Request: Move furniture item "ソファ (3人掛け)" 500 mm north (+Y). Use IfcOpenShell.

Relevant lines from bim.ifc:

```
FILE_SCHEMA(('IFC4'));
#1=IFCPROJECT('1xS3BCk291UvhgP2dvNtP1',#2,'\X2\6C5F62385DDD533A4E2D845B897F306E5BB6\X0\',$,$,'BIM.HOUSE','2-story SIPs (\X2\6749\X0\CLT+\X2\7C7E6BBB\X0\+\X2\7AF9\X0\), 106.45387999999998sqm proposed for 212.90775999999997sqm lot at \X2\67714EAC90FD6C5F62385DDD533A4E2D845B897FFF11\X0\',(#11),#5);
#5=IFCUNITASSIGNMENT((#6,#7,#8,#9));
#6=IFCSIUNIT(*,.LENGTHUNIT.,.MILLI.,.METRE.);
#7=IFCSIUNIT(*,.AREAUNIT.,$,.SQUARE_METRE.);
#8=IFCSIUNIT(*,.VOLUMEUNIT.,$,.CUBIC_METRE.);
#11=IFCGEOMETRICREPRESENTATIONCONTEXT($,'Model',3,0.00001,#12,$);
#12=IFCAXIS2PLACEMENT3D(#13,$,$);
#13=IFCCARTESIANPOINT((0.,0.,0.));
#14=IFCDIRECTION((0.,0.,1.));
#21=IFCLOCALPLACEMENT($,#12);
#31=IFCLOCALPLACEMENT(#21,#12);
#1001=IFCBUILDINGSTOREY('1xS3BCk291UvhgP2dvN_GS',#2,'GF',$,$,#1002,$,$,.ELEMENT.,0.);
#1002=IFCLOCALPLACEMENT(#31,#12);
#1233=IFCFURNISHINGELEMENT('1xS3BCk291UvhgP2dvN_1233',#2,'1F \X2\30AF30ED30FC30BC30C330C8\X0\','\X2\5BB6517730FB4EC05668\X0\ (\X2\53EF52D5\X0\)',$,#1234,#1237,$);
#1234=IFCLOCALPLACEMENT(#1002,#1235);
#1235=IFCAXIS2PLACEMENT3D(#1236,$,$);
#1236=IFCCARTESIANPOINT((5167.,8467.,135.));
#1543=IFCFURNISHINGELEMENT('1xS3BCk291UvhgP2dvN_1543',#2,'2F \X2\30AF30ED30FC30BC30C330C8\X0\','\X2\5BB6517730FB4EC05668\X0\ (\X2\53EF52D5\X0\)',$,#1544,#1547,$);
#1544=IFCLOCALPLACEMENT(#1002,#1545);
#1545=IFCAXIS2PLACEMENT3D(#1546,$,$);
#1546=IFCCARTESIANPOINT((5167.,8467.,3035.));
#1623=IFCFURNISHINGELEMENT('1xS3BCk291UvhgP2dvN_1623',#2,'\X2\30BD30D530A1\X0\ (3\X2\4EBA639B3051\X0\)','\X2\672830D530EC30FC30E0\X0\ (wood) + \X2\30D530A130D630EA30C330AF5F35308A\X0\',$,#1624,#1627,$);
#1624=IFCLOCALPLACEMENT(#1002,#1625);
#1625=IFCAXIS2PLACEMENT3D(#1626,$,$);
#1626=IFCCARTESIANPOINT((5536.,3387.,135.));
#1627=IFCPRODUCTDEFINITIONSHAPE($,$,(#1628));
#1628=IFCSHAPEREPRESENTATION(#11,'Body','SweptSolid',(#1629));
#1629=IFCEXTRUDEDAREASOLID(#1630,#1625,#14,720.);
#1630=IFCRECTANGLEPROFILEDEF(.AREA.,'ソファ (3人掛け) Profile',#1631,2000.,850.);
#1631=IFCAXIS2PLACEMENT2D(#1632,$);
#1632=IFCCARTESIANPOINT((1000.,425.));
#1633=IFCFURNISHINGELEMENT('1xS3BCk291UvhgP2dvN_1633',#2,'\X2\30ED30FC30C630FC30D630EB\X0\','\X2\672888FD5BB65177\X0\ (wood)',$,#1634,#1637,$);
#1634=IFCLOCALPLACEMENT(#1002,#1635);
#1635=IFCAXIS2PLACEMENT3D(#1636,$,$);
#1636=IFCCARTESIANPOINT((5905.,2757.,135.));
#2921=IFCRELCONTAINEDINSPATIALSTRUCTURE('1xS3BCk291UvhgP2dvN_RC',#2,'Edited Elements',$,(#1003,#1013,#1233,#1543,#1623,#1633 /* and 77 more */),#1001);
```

```python
import ifcopenshell
import ifcopenshell.api.geometry
import ifcopenshell.util.placement

model = ifcopenshell.open("bim.ifc")

item = model.by_guid("1xS3BCk291UvhgP2dvN_1623")
matrix = ifcopenshell.util.placement.get_local_placement(item.ObjectPlacement)
matrix[1, 3] += 500.0
ifcopenshell.api.geometry.edit_object_placement(model, product=item, matrix=matrix, is_si=False)

print(ifcopenshell.util.placement.get_local_placement(item.ObjectPlacement).round(3) + 0.0)

model.write("bim_v2.ifc")
```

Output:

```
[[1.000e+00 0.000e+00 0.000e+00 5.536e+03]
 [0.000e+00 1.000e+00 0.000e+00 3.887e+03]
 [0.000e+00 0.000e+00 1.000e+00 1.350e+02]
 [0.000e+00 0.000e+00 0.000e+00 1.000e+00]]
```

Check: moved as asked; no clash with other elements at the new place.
